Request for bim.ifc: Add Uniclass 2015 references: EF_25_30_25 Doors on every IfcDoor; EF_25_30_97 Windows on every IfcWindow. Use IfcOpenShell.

First a look at what the model holds.

```python
import ifcopenshell

model = ifcopenshell.open("bim.ifc")
print(model.schema)
print("classifications:", [c.Name for c in model.by_type("IfcClassification")])
for ifc_class in ("IfcDoor", "IfcRoof", "IfcStair", "IfcWall", "IfcWindow"):
    print(ifc_class, len(model.by_type(ifc_class)))
```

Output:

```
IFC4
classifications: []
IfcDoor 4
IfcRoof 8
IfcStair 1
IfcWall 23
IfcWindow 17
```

```python
import ifcopenshell
import ifcopenshell.api.classification

model = ifcopenshell.open("bim.ifc")

system = ifcopenshell.api.classification.add_classification(model, classification="Uniclass 2015")

codes = {
    "IfcDoor": ("EF_25_30_25", "Doors"),
    "IfcWindow": ("EF_25_30_97", "Windows"),
}
for ifc_class, (code, name) in codes.items():
    products = model.by_type(ifc_class)
    ifcopenshell.api.classification.add_reference(
        model, products=products, classification=system, identification=code, name=name
    )
    print(code, len(products))

model.write("bim-out.ifc")
```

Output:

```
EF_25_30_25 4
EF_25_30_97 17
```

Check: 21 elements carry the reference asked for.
